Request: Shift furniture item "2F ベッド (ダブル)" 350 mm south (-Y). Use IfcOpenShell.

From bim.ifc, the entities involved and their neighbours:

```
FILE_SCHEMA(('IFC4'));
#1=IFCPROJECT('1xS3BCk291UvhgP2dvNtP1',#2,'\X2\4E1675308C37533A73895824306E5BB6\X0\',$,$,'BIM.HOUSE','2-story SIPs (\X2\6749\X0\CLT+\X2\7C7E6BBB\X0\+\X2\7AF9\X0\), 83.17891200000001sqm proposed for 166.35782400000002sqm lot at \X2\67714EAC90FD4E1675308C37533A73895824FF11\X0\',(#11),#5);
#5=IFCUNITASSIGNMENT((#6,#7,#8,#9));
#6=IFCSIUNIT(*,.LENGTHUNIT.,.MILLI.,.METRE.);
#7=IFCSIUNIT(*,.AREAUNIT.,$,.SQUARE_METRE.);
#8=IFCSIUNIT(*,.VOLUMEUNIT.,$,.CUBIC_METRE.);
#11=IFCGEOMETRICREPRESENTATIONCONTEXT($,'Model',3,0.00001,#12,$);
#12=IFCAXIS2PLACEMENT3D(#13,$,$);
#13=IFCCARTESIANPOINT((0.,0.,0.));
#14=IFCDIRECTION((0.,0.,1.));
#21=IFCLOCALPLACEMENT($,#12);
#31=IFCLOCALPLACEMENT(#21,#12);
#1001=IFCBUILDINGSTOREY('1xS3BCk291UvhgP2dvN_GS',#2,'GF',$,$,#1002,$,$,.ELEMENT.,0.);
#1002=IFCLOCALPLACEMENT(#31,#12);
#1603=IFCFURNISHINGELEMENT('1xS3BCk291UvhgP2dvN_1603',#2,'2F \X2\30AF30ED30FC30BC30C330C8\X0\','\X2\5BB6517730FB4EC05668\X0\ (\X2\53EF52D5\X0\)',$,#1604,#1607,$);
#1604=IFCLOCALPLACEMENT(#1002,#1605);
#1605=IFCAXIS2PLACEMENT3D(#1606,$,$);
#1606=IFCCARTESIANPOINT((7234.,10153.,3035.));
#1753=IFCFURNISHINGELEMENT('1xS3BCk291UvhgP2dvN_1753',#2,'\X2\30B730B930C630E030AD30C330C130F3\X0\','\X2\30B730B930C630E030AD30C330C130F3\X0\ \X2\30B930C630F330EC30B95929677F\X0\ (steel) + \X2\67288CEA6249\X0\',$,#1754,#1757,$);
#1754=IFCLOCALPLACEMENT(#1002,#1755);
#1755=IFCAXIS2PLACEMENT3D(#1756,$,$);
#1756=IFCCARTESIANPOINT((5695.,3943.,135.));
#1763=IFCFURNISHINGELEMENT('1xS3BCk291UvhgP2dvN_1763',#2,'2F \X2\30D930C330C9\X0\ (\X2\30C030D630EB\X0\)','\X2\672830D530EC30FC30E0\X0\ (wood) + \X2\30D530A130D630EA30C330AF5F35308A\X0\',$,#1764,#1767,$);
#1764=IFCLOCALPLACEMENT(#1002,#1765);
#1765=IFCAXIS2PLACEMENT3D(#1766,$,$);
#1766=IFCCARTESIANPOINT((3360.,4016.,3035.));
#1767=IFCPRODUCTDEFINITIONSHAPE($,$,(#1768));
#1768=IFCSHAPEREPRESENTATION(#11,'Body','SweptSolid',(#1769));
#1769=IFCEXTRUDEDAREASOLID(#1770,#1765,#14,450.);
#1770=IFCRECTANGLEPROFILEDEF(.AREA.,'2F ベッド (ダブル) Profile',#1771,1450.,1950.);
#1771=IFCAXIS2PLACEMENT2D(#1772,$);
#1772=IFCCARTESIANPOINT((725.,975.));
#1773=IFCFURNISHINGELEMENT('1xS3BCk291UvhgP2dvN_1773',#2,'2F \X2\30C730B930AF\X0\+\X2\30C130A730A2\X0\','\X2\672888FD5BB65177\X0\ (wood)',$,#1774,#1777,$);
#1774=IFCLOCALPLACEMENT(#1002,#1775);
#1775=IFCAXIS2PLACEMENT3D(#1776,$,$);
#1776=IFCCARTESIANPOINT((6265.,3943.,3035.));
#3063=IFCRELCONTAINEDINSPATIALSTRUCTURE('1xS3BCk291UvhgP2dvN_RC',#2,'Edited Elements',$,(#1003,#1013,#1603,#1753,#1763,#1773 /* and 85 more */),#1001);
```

```python
import ifcopenshell
import ifcopenshell.api.geometry
import ifcopenshell.util.placement
import ifcopenshell.util.unit

model = ifcopenshell.open("bim.ifc")
unit_scale = ifcopenshell.util.unit.calculate_unit_scale(model)

item = model.by_guid("1xS3BCk291UvhgP2dvN_1763")
matrix = ifcopenshell.util.placement.get_local_placement(item.ObjectPlacement)
matrix[1, 3] -= 0.35 / unit_scale
ifcopenshell.api.geometry.edit_object_placement(model, product=item, matrix=matrix, is_si=False)

print(ifcopenshell.util.placement.get_local_placement(item.ObjectPlacement).round(3) + 0.0)

model.write("bim_rev.ifc")
```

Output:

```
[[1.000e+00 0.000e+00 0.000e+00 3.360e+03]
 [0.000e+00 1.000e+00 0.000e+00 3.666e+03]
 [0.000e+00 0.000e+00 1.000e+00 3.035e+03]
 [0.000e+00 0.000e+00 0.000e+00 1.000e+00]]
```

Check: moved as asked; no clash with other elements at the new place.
